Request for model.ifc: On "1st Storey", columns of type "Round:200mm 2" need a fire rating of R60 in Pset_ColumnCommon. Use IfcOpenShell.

First a look at what the model holds.

```python
import ifcopenshell
import ifcopenshell.util.element

model = ifcopenshell.open("model.ifc")
print(model.schema)
storey = next(s for s in model.by_type("IfcBuildingStorey") if s.Name == "1st Storey")
columns = [e for e in ifcopenshell.util.element.get_decomposition(storey) if e.is_a("IfcColumn")]
seen = {}
for e in columns:
    element_type = ifcopenshell.util.element.get_type(e)
    key = (element_type.Name if element_type != e and element_type else None, ifcopenshell.util.element.get_pset(e, "Pset_ColumnCommon", "FireRating"))
    seen[key] = seen.get(key, 0) + 1
for (name, value), count in sorted(seen.items(), key=str):
    print(count, "x", name, "|", value)
```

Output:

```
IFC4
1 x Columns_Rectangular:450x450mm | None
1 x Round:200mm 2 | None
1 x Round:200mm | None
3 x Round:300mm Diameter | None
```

```python
import ifcopenshell
import ifcopenshell.api.pset
import ifcopenshell.util.element

model = ifcopenshell.open("model.ifc")

storey = next(s for s in model.by_type("IfcBuildingStorey") if s.Name == "1st Storey")
columns = [e for e in ifcopenshell.util.element.get_decomposition(storey) if e.is_a("IfcColumn")]

count = 0
for e in columns:
    element_type = ifcopenshell.util.element.get_type(e)
    if element_type in (None, e) or element_type.Name != "Round:200mm 2":
        continue
    # add_pset returns the element's existing set when there is one.
    pset = ifcopenshell.api.pset.add_pset(model, product=e, name="Pset_ColumnCommon")
    ifcopenshell.api.pset.edit_pset(model, pset=pset, properties={"FireRating": "R60"})
    count += 1

print(count, "columns updated")

model.write("model_edited.ifc")
```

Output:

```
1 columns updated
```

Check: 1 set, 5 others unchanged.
